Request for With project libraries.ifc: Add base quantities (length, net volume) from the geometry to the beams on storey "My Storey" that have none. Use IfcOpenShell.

First a look at what the model holds.

```python
import ifcopenshell
import ifcopenshell.util.element
import ifcopenshell.util.unit

model = ifcopenshell.open("With project libraries.ifc")
print(model.schema)
for unit_type in ("LENGTHUNIT", "AREAUNIT", "VOLUMEUNIT"):
    print(unit_type, ifcopenshell.util.unit.calculate_unit_scale(model, unit_type))
storey = next(s for s in model.by_type("IfcBuildingStorey") if s.Name == "My Storey")
beams = [e for e in ifcopenshell.util.element.get_decomposition(storey) if e.is_a("IfcBeam")]
for e in sorted(beams, key=lambda e: e.id()):
    print(e.id(), e.is_a(), e.Name, list(ifcopenshell.util.element.get_psets(e, qtos_only=True)), sep=" | ")
```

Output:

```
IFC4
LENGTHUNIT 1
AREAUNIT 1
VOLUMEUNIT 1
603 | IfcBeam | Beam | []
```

```python
import ifcopenshell
import ifcopenshell.api.pset
import ifcopenshell.geom
import ifcopenshell.util.element
import ifcopenshell.util.shape
import ifcopenshell.util.unit

model = ifcopenshell.open("With project libraries.ifc")
unit_scale = ifcopenshell.util.unit.calculate_unit_scale(model)
volume_scale = ifcopenshell.util.unit.calculate_unit_scale(model, "VOLUMEUNIT")
settings = ifcopenshell.geom.settings()

storey = next(s for s in model.by_type("IfcBuildingStorey") if s.Name == "My Storey")
beams = [e for e in ifcopenshell.util.element.get_decomposition(storey) if e.is_a("IfcBeam")]

for e in sorted(beams, key=lambda e: e.id()):
    if ifcopenshell.util.element.get_psets(e, qtos_only=True, should_inherit=False):
        continue
    # Geometry comes back in metres, in the element's own axes.
    shape = ifcopenshell.geom.create_shape(settings, e)
    values = {
        "Length": ifcopenshell.util.shape.get_max_xyz(shape.geometry) / unit_scale,
        "NetVolume": ifcopenshell.util.shape.get_volume(shape.geometry) / volume_scale,
    }
    qto = ifcopenshell.api.pset.add_qto(model, product=e, name="Qto_BeamBaseQuantities")
    ifcopenshell.api.pset.edit_qto(model, qto=qto, properties=values)
    print(e.id(), {k: round(v, 3) for k, v in values.items()})

model.write("With project libraries-out.ifc")
```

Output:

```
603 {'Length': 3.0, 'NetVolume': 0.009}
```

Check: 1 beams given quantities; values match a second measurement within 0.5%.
